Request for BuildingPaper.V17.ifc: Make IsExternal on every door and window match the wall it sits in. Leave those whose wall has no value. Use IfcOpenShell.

First a look at what the model holds.

```python
import ifcopenshell
import ifcopenshell.util.element

model = ifcopenshell.open("BuildingPaper.V17.ifc")
print(model.schema)
seen = {}
for e in model.by_type("IfcDoor") + model.by_type("IfcWindow"):
    if not e.FillsVoids:
        continue
    host = e.FillsVoids[0].RelatingOpeningElement.VoidsElements[0].RelatingBuildingElement
    own = ifcopenshell.util.element.get_pset(e, f"Pset_{e.is_a()[3:].removesuffix('StandardCase')}Common", "IsExternal")
    wall = ifcopenshell.util.element.get_pset(host, "Pset_WallCommon", "IsExternal")
    seen[e.is_a(), own, wall] = seen.get((e.is_a(), own, wall), 0) + 1
for (cls, own, wall), count in sorted(seen.items(), key=str):
    print(count, cls, "IsExternal:", own, "| host wall:", wall)
```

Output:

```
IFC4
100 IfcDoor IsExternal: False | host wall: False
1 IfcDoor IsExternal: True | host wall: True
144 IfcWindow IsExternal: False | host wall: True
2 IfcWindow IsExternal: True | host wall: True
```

```python
import ifcopenshell
import ifcopenshell.api.pset
import ifcopenshell.util.element

model = ifcopenshell.open("BuildingPaper.V17.ifc")

count = 0
for ifc_class, pset_name in (("IfcDoor", "Pset_DoorCommon"), ("IfcWindow", "Pset_WindowCommon")):
    for e in model.by_type(ifc_class):
        if not e.FillsVoids:
            continue
        host = e.FillsVoids[0].RelatingOpeningElement.VoidsElements[0].RelatingBuildingElement
        external = ifcopenshell.util.element.get_pset(host, "Pset_WallCommon", "IsExternal")
        if external is None or ifcopenshell.util.element.get_pset(e, pset_name, "IsExternal") == external:
            continue
        pset = ifcopenshell.api.pset.add_pset(model, product=e, name=pset_name)
        ifcopenshell.api.pset.edit_pset(model, pset=pset, properties={"IsExternal": external})
        count += 1

print(count, "updated")

model.write("BuildingPaper.V17_v2.ifc")
```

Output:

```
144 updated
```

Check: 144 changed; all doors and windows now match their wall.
